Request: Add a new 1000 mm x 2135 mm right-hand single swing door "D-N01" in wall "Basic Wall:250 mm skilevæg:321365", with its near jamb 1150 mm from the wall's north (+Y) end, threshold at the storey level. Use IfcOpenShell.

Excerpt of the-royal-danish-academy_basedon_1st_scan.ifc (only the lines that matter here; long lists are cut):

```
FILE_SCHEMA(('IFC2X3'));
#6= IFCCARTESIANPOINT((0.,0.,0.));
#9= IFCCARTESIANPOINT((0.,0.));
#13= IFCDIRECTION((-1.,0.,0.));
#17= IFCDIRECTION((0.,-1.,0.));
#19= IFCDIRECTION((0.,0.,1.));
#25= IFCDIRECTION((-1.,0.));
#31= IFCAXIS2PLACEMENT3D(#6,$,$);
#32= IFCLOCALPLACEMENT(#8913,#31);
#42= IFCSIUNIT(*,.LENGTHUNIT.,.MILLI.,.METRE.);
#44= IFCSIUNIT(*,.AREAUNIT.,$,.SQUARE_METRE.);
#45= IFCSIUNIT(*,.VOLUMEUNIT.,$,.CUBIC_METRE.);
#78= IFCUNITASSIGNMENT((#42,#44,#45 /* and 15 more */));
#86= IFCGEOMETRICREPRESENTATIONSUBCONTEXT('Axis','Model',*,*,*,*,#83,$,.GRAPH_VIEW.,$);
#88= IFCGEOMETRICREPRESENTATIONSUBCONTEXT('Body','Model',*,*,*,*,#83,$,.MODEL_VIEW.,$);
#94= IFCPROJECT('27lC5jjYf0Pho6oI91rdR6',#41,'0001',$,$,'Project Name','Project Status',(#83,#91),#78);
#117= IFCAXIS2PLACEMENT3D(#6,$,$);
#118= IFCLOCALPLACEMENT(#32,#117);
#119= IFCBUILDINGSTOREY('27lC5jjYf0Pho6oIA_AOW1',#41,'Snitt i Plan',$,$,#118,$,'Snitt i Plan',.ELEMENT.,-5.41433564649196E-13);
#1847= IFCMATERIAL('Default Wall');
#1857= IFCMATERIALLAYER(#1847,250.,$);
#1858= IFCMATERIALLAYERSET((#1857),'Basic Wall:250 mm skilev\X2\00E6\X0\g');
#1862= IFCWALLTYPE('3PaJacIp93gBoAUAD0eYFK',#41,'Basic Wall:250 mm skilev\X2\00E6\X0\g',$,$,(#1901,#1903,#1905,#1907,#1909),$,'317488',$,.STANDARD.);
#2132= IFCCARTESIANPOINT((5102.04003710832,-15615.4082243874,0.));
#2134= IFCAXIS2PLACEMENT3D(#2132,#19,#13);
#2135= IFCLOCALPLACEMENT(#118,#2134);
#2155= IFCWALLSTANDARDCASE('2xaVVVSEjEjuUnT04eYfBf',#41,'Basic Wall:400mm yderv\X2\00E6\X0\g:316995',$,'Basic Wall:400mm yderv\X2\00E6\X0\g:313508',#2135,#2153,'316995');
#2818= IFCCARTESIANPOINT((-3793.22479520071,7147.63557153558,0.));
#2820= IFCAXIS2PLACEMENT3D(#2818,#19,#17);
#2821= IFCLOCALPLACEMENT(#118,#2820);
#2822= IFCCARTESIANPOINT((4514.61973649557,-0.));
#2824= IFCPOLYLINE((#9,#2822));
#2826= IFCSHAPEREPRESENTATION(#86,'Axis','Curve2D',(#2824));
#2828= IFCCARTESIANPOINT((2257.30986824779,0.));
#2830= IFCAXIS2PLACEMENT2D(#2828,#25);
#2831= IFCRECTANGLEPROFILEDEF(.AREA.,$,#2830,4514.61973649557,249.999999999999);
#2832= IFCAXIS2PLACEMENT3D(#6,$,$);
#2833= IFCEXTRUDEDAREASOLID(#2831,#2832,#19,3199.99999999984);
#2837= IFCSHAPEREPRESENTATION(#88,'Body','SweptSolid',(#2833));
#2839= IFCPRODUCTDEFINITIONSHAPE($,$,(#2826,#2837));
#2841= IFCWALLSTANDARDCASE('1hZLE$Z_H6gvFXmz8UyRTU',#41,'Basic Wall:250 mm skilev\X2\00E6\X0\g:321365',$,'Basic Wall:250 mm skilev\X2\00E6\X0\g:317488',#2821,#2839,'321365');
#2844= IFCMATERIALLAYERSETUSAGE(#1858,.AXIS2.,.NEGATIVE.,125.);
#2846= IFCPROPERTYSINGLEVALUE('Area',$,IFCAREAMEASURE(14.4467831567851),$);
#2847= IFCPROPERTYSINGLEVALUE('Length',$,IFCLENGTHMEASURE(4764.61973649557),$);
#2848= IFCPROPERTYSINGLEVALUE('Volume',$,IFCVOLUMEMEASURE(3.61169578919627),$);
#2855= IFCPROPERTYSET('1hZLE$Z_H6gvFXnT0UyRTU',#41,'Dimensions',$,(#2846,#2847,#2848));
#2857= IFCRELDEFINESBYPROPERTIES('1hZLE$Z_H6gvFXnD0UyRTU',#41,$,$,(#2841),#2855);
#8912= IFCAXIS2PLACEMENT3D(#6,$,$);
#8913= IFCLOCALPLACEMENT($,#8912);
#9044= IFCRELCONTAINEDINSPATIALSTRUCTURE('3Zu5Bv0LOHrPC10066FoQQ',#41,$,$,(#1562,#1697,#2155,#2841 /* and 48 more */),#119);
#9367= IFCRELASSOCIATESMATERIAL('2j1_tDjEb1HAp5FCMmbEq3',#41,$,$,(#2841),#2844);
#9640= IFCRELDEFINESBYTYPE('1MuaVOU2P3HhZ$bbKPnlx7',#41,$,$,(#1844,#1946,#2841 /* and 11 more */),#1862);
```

```python
import numpy as np
import ifcopenshell
import ifcopenshell.api.feature
import ifcopenshell.api.geometry
import ifcopenshell.api.pset
import ifcopenshell.api.root
import ifcopenshell.api.spatial
import ifcopenshell.api.type
import ifcopenshell.geom
import ifcopenshell.util.element
import ifcopenshell.util.placement
import ifcopenshell.util.representation
import ifcopenshell.util.shape
import ifcopenshell.util.unit

model = ifcopenshell.open("the-royal-danish-academy_basedon_1st_scan.ifc")
unit_scale = ifcopenshell.util.unit.calculate_unit_scale(model)
area_scale = ifcopenshell.util.unit.calculate_unit_scale(model, "AREAUNIT")
volume_scale = ifcopenshell.util.unit.calculate_unit_scale(model, "VOLUMEUNIT")
settings = ifcopenshell.geom.settings()


def volume(element):
    """Net volume in cubic metres, openings subtracted."""
    shape = ifcopenshell.geom.create_shape(settings, element)
    return ifcopenshell.util.shape.get_volume(shape.geometry)


wall = model.by_guid("1hZLE$Z_H6gvFXmz8UyRTU")
storey = ifcopenshell.util.element.get_container(wall, ifc_class="IfcBuildingStorey")
context = ifcopenshell.util.representation.get_context(model, "Model", "Body", "MODEL_VIEW")
before = volume(wall)

width, height, from_end, sill = 1, 2.135, 1.15, 0.0  # metres

# The wall runs along its own X axis, and the end named is its -X end.
wall_shape = ifcopenshell.geom.create_shape(settings, wall)
x, y, z = ifcopenshell.util.shape.get_vertices(wall_shape.geometry).T
start = x.min() + from_end
face, thickness = float(y.min()), float(y.max() - y.min())
wall_matrix = ifcopenshell.util.placement.get_local_placement(wall.ObjectPlacement)
level = ifcopenshell.util.placement.get_local_placement(storey.ObjectPlacement)[2, 3]


def in_wall(x, y):
    """Placement at x, y metres in the wall's axes, at sill height."""
    matrix = wall_matrix.copy()
    matrix[:, 3] = wall_matrix @ np.array([x / unit_scale, y / unit_scale, 0.0, 1.0])
    matrix[2, 3] = level + sill / unit_scale
    return matrix


# Opening: a box that overshoots both wall faces by 50 mm.
opening = ifcopenshell.api.root.create_entity(model, ifc_class="IfcOpeningElement")
box = ifcopenshell.api.geometry.add_wall_representation(
    model, context=context, length=width, height=height, thickness=thickness + 0.1
)
ifcopenshell.api.geometry.assign_representation(model, product=opening, representation=box)
ifcopenshell.api.geometry.edit_object_placement(model, product=opening, matrix=in_wall(start, face - 0.05), is_si=False)
ifcopenshell.api.feature.add_feature(model, feature=opening, element=wall)

door = ifcopenshell.api.root.create_entity(model, ifc_class="IfcDoor", name="D-N01")
door.OverallWidth, door.OverallHeight = width / unit_scale, height / unit_scale
body = ifcopenshell.api.geometry.add_door_representation(
    model,
    context=context,
    overall_width=door.OverallWidth,
    overall_height=door.OverallHeight,
    operation_type="SINGLE_SWING_RIGHT",
    lining_properties={"LiningDepth": thickness / unit_scale, "ThresholdDepth": thickness / unit_scale},
)
ifcopenshell.api.geometry.assign_representation(model, product=door, representation=body)
ifcopenshell.api.spatial.assign_container(model, products=[door], relating_structure=storey)
fills = ifcopenshell.api.feature.add_filling(model, opening=opening, element=door)
fills.OwnerHistory = door.OwnerHistory  # required in IFC2X3

# IFC2X3 keeps the operation on the door style.
style = ifcopenshell.api.root.create_entity(model, ifc_class="IfcDoorStyle", name="D-N01")
style.OperationType, style.ConstructionType = "SINGLE_SWING_RIGHT", "NOTDEFINED"
style.ParameterTakesPrecedence = style.Sizeable = False
ifcopenshell.api.type.assign_type(model, related_objects=[door], relating_type=style)

# The lining spans the wall, so the door starts at the wall face.
ifcopenshell.api.geometry.edit_object_placement(model, product=door, matrix=in_wall(start, face), is_si=False)

after = volume(wall)

# Update the wall's stored quantities.
pset = model.by_id(ifcopenshell.util.element.get_pset(wall, "Dimensions", should_inherit=False)["id"])
ifcopenshell.api.pset.edit_pset(model, pset=pset, properties={
    "Area": model.create_entity("IfcAreaMeasure", after / thickness / area_scale),
    "Volume": model.create_entity("IfcVolumeMeasure", after / volume_scale),
})

print(f"wall volume {before:.3f} -> {after:.3f} m3")

model.write("the-royal-danish-academy_basedon_1st_scan_rev.ifc")
```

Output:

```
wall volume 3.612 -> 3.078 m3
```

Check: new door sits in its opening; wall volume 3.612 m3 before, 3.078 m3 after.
